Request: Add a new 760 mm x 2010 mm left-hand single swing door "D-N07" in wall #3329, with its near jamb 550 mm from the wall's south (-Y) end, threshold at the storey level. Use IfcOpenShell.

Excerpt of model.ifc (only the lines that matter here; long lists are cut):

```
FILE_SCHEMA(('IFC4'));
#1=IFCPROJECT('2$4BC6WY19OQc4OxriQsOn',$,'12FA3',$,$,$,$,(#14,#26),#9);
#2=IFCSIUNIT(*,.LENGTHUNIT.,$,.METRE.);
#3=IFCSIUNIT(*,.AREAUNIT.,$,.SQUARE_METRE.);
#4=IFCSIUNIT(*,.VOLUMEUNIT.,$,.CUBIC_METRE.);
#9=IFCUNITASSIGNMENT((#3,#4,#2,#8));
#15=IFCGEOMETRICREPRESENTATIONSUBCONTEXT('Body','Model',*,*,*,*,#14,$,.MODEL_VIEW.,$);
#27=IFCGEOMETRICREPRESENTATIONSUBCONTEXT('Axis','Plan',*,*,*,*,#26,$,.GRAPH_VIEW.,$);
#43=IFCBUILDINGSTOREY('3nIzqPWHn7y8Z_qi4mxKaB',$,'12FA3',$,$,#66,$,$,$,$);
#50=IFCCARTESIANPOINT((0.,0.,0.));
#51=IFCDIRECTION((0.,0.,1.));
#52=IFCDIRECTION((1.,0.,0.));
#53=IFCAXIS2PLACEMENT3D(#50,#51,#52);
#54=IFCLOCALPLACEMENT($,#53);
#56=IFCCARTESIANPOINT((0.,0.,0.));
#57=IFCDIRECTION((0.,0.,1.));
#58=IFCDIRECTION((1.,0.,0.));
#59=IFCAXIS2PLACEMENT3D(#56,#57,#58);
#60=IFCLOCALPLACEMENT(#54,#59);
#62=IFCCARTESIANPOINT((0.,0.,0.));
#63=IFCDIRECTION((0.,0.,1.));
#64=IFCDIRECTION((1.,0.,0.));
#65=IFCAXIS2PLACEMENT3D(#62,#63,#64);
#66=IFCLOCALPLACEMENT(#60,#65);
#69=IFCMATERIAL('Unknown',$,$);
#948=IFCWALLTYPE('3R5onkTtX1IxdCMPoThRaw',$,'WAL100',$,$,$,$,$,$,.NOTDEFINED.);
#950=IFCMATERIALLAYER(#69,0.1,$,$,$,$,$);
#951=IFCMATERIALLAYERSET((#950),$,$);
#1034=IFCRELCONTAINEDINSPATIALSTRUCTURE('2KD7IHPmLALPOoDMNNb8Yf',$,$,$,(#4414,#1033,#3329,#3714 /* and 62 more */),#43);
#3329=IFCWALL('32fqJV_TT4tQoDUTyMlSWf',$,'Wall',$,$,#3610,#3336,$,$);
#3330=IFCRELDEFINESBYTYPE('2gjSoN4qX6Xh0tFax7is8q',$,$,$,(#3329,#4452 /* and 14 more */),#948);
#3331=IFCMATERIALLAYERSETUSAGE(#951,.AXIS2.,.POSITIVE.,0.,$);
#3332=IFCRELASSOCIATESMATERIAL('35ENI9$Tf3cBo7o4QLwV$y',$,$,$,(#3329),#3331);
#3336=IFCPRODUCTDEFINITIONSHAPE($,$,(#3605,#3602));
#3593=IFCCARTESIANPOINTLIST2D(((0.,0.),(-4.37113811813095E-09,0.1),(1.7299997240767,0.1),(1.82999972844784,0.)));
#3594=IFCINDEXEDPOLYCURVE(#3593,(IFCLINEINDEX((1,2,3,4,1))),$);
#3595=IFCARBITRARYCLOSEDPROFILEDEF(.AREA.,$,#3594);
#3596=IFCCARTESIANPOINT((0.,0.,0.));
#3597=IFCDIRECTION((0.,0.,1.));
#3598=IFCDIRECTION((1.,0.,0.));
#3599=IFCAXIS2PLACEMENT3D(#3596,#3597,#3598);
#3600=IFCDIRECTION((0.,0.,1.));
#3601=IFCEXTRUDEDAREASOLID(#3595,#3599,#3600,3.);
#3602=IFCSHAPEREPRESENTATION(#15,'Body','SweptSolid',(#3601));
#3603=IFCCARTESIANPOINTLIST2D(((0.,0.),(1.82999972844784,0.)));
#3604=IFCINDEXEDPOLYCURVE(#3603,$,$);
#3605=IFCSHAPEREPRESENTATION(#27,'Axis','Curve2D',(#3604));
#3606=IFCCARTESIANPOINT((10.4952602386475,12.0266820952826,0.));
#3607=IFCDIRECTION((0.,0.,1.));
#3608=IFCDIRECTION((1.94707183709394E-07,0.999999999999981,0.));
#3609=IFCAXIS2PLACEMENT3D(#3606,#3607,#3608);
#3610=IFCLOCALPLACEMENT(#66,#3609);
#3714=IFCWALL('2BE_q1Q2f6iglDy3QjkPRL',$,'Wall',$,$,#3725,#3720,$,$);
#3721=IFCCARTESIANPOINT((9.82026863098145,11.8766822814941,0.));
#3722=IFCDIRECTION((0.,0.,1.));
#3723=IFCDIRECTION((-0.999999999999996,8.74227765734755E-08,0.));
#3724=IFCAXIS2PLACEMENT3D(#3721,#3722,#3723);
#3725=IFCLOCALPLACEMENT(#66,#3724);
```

```python
import numpy as np
import ifcopenshell
import ifcopenshell.api.feature
import ifcopenshell.api.geometry
import ifcopenshell.api.root
import ifcopenshell.api.spatial
import ifcopenshell.geom
import ifcopenshell.util.element
import ifcopenshell.util.placement
import ifcopenshell.util.representation
import ifcopenshell.util.shape
import ifcopenshell.util.unit

model = ifcopenshell.open("model.ifc")
unit_scale = ifcopenshell.util.unit.calculate_unit_scale(model)
settings = ifcopenshell.geom.settings()


def volume(element):
    """Net volume in cubic metres, openings subtracted."""
    shape = ifcopenshell.geom.create_shape(settings, element)
    return ifcopenshell.util.shape.get_volume(shape.geometry)


wall = model.by_guid("32fqJV_TT4tQoDUTyMlSWf")
storey = ifcopenshell.util.element.get_container(wall, ifc_class="IfcBuildingStorey")
context = ifcopenshell.util.representation.get_context(model, "Model", "Body", "MODEL_VIEW")
before = volume(wall)

width, height, from_end, sill = 0.76, 2.01, 0.55, 0.0  # metres

# The wall runs along its own X axis, and the end named is its -X end.
wall_shape = ifcopenshell.geom.create_shape(settings, wall)
x, y, z = ifcopenshell.util.shape.get_vertices(wall_shape.geometry).T
start = x.min() + from_end
face, thickness = float(y.min()), float(y.max() - y.min())
wall_matrix = ifcopenshell.util.placement.get_local_placement(wall.ObjectPlacement)
level = ifcopenshell.util.placement.get_local_placement(storey.ObjectPlacement)[2, 3]


def in_wall(x, y):
    """Placement at x, y metres in the wall's axes, at sill height."""
    matrix = wall_matrix.copy()
    matrix[:, 3] = wall_matrix @ np.array([x / unit_scale, y / unit_scale, 0.0, 1.0])
    matrix[2, 3] = level + sill / unit_scale
    return matrix


# Opening: a box that overshoots both wall faces by 50 mm.
opening = ifcopenshell.api.root.create_entity(model, ifc_class="IfcOpeningElement", predefined_type="OPENING")
box = ifcopenshell.api.geometry.add_wall_representation(
    model, context=context, length=width, height=height, thickness=thickness + 0.1
)
ifcopenshell.api.geometry.assign_representation(model, product=opening, representation=box)
ifcopenshell.api.geometry.edit_object_placement(model, product=opening, matrix=in_wall(start, face - 0.05), is_si=False)
ifcopenshell.api.feature.add_feature(model, feature=opening, element=wall)

door = ifcopenshell.api.root.create_entity(model, ifc_class="IfcDoor", name="D-N07", predefined_type="DOOR")
door.OverallWidth, door.OverallHeight = width / unit_scale, height / unit_scale
door.OperationType = "SINGLE_SWING_LEFT"
body = ifcopenshell.api.geometry.add_door_representation(
    model,
    context=context,
    overall_width=door.OverallWidth,
    overall_height=door.OverallHeight,
    operation_type="SINGLE_SWING_LEFT",
    lining_properties={"LiningDepth": thickness / unit_scale, "ThresholdDepth": thickness / unit_scale},
)
ifcopenshell.api.geometry.assign_representation(model, product=door, representation=body)
ifcopenshell.api.spatial.assign_container(model, products=[door], relating_structure=storey)
ifcopenshell.api.feature.add_filling(model, opening=opening, element=door)

# The lining spans the wall, so the door starts at the wall face.
ifcopenshell.api.geometry.edit_object_placement(model, product=door, matrix=in_wall(start, face), is_si=False)

after = volume(wall)

print(f"wall volume {before:.3f} -> {after:.3f} m3")

model.write("model_updated.ifc")
```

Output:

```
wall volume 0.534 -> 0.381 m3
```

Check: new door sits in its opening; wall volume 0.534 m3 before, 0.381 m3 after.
